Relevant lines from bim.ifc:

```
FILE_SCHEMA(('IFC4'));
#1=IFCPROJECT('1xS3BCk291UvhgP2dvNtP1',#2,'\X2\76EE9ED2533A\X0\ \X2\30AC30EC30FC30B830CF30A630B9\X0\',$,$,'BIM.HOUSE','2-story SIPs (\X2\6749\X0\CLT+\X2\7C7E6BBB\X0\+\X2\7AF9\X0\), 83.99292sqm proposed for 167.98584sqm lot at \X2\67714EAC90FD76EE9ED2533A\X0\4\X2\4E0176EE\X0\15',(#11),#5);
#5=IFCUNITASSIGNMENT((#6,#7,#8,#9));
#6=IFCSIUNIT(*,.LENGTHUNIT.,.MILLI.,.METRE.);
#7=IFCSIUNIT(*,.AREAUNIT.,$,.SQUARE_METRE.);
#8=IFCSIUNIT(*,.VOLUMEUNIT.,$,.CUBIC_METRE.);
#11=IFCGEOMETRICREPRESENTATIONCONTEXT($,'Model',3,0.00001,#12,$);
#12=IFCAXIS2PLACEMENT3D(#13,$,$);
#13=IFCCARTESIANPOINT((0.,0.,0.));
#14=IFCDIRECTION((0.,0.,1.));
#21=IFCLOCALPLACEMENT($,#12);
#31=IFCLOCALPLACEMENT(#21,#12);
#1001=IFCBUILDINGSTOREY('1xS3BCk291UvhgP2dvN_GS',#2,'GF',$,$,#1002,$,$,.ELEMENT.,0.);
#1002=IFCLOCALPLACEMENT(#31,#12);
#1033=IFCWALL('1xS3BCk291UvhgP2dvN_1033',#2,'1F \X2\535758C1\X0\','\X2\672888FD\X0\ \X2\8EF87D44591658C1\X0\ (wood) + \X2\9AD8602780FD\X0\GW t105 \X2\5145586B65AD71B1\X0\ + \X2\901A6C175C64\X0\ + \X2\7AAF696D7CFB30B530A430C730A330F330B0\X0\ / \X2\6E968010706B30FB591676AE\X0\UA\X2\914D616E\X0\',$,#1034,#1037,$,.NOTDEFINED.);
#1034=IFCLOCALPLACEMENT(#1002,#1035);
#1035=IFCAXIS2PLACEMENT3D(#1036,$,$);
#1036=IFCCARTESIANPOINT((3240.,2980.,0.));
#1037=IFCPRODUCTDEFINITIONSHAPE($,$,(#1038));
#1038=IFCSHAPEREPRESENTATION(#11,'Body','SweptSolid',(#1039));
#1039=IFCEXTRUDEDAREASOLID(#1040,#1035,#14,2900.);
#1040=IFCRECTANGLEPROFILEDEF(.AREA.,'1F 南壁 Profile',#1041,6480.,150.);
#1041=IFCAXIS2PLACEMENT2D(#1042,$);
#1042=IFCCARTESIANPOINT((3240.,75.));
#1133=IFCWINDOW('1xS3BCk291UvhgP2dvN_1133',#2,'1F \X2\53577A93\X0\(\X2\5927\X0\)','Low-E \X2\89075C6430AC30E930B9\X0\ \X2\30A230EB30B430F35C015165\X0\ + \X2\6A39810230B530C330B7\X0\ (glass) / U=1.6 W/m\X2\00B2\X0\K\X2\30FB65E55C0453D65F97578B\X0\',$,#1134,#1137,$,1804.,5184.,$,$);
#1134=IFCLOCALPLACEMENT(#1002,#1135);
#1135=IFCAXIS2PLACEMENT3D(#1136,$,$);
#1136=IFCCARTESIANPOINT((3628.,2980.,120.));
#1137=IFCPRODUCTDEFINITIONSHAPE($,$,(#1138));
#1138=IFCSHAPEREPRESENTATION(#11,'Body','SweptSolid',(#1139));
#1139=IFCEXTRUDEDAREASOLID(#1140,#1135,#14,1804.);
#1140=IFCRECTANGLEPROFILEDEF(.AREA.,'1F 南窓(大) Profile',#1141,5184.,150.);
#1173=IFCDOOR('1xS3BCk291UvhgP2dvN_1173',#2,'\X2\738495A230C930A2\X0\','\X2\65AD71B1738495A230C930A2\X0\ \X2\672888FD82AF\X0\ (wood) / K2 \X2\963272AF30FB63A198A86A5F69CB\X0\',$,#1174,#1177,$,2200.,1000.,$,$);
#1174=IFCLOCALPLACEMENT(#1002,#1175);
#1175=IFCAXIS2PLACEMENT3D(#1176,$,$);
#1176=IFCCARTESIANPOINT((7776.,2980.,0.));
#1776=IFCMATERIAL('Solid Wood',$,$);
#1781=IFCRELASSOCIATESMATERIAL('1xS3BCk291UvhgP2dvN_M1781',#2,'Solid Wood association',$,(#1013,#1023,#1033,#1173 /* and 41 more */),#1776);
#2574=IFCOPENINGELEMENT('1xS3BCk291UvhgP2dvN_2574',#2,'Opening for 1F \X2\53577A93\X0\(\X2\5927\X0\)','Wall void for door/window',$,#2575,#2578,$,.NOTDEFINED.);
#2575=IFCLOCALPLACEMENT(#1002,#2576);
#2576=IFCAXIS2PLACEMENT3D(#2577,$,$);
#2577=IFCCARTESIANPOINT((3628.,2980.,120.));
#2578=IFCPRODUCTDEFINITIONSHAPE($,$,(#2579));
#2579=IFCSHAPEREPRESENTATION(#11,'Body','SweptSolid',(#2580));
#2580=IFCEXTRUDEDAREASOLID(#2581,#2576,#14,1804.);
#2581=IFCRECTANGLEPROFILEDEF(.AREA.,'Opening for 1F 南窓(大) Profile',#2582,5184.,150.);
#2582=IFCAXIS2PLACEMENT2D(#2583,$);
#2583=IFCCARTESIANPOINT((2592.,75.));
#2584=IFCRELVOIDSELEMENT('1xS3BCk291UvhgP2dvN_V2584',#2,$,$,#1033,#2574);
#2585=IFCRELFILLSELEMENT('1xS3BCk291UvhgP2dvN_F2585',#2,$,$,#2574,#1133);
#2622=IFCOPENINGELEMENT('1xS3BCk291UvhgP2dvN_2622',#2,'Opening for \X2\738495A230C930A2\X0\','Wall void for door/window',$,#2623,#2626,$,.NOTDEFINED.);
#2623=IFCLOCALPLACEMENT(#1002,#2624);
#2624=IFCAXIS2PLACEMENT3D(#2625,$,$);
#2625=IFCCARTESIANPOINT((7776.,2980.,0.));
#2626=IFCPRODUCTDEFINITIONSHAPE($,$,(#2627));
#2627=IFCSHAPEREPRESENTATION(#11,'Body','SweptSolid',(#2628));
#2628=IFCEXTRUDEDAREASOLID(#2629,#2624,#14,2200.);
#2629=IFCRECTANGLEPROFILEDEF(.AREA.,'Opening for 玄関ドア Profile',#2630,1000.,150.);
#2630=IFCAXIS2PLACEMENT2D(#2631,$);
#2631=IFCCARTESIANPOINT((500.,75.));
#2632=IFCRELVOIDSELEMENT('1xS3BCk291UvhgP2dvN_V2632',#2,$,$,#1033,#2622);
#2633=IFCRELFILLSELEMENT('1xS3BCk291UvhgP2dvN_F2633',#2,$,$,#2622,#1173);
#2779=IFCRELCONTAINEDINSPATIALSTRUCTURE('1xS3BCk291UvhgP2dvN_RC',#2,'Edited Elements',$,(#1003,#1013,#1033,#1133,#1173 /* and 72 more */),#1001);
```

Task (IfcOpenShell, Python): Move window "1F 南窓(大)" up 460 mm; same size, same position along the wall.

```python
import numpy as np
import ifcopenshell
import ifcopenshell.api.geometry
import ifcopenshell.util.placement
import ifcopenshell.util.unit

model = ifcopenshell.open("bim.ifc")
unit_scale = ifcopenshell.util.unit.calculate_unit_scale(model)

window = model.by_guid("1xS3BCk291UvhgP2dvN_1133")
opening = window.FillsVoids[0].RelatingOpeningElement
dz = 0.46 / unit_scale

shift = np.array([0.0, 0.0, dz])
# The window is not placed relative to its opening, so move both.
for product in (opening, window):
    matrix = ifcopenshell.util.placement.get_local_placement(product.ObjectPlacement)
    matrix[:3, 3] += shift
    ifcopenshell.api.geometry.edit_object_placement(model, product=product, matrix=matrix, is_si=False)

print(f"moved by {dz * unit_scale:+.3f} m")

model.write("bim_updated.ifc")
```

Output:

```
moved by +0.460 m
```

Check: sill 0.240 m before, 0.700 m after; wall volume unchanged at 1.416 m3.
